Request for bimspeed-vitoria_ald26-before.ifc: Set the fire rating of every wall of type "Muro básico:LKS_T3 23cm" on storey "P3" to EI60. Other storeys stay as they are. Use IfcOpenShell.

First a look at what the model holds.

```python
import ifcopenshell
import ifcopenshell.util.element

model = ifcopenshell.open("bimspeed-vitoria_ald26-before.ifc")
print(model.schema)
storey = next(s for s in model.by_type("IfcBuildingStorey") if s.Name == "P3")
walls = [e for e in ifcopenshell.util.element.get_decomposition(storey) if e.is_a("IfcWall")]
seen = {}
for e in walls:
    element_type = ifcopenshell.util.element.get_type(e)
    key = (element_type.Name if element_type != e and element_type else None, ifcopenshell.util.element.get_pset(e, "Pset_WallCommon", "FireRating"))
    seen[key] = seen.get(key, 0) + 1
for (name, value), count in sorted(seen.items(), key=str):
    print(count, "x", name, "|", value)
```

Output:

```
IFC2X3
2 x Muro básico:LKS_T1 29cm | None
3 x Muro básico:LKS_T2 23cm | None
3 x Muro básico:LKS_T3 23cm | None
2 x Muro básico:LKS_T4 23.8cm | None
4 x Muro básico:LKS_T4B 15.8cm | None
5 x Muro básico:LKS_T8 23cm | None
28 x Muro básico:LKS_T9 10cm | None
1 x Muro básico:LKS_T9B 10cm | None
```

```python
import ifcopenshell
import ifcopenshell.api.pset
import ifcopenshell.util.element

model = ifcopenshell.open("bimspeed-vitoria_ald26-before.ifc")

storey = next(s for s in model.by_type("IfcBuildingStorey") if s.Name == "P3")
walls = [e for e in ifcopenshell.util.element.get_decomposition(storey) if e.is_a("IfcWall")]

count = 0
for e in walls:
    element_type = ifcopenshell.util.element.get_type(e)
    if element_type in (None, e) or element_type.Name != "Muro básico:LKS_T3 23cm":
        continue
    # add_pset returns the element's existing set when there is one.
    pset = ifcopenshell.api.pset.add_pset(model, product=e, name="Pset_WallCommon")
    ifcopenshell.api.pset.edit_pset(model, pset=pset, properties={"FireRating": "EI60"})
    count += 1

print(count, "walls updated")

model.write("bimspeed-vitoria_ald26-before_v2.ifc")
```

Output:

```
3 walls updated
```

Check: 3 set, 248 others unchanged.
